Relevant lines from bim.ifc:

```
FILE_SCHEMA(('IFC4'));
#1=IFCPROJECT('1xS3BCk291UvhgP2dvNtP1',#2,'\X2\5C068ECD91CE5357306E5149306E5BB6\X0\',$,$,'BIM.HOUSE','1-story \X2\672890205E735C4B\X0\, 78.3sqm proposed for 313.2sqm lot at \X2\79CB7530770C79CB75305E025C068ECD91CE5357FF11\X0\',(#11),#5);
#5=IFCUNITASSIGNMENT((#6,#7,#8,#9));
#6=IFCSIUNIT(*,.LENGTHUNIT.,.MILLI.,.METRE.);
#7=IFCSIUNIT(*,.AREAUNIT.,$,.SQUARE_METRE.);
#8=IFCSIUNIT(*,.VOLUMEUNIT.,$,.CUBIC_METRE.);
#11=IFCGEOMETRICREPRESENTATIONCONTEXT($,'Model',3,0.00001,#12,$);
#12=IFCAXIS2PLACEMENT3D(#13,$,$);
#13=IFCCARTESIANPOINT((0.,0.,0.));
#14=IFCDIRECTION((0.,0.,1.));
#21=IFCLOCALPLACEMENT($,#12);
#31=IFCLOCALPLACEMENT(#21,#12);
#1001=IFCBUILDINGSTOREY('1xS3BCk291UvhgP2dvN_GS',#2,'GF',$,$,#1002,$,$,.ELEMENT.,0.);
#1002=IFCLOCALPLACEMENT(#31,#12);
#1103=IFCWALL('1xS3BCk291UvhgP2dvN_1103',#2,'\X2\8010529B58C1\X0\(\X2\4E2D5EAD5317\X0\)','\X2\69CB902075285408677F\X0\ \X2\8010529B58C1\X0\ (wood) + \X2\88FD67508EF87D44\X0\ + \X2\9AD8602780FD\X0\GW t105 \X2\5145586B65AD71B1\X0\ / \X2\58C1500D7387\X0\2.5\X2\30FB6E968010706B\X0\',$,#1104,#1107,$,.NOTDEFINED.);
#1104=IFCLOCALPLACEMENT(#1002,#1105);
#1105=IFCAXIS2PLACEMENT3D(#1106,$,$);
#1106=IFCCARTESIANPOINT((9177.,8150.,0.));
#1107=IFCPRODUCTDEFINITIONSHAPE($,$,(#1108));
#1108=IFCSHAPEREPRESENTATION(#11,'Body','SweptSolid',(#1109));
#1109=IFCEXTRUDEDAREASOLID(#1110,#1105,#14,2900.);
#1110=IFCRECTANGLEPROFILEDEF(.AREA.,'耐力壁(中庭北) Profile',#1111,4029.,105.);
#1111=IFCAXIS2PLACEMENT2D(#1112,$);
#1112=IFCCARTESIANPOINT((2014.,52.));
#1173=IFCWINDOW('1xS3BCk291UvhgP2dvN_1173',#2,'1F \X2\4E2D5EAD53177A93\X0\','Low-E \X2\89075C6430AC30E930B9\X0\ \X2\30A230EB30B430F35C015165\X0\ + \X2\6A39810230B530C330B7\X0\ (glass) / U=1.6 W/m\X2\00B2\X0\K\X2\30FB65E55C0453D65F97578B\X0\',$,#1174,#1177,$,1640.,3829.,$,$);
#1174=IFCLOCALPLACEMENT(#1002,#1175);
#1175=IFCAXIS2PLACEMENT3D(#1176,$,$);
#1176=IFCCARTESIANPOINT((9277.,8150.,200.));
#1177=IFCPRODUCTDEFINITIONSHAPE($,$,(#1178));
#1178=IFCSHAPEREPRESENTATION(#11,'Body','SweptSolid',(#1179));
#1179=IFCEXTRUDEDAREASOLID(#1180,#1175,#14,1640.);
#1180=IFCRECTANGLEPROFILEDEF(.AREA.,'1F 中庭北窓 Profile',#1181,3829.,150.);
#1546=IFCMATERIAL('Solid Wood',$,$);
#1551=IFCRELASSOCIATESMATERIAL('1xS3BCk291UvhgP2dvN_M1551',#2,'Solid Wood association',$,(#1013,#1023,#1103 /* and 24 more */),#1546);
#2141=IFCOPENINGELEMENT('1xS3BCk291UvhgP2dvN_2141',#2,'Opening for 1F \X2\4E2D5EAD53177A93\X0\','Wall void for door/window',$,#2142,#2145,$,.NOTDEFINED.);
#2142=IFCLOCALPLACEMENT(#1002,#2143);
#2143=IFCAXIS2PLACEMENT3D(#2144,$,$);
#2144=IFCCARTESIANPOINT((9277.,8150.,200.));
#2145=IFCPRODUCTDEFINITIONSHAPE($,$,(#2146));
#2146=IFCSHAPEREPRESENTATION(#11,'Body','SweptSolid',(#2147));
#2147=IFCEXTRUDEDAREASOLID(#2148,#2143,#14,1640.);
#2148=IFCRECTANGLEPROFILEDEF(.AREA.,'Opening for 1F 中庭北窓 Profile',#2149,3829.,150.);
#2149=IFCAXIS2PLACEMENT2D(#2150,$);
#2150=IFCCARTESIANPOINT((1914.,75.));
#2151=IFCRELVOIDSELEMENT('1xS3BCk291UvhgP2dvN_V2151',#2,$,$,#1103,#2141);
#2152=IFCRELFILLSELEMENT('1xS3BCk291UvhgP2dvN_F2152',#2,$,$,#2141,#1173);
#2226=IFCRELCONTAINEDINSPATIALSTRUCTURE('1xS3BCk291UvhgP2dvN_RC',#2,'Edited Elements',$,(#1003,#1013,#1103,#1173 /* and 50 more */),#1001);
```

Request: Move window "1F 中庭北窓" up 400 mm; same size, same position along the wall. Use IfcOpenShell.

```python
import numpy as np
import ifcopenshell
import ifcopenshell.api.geometry
import ifcopenshell.util.placement
import ifcopenshell.util.unit

model = ifcopenshell.open("bim.ifc")
unit_scale = ifcopenshell.util.unit.calculate_unit_scale(model)

window = model.by_guid("1xS3BCk291UvhgP2dvN_1173")
opening = window.FillsVoids[0].RelatingOpeningElement
dz = 0.4 / unit_scale

shift = np.array([0.0, 0.0, dz])
# The window is not placed relative to its opening, so move both.
for product in (opening, window):
    matrix = ifcopenshell.util.placement.get_local_placement(product.ObjectPlacement)
    matrix[:3, 3] += shift
    ifcopenshell.api.geometry.edit_object_placement(model, product=product, matrix=matrix, is_si=False)

print(f"moved by {dz * unit_scale:+.3f} m")

model.write("bim_updated.ifc")
```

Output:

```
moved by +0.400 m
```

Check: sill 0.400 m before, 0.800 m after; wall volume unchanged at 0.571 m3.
